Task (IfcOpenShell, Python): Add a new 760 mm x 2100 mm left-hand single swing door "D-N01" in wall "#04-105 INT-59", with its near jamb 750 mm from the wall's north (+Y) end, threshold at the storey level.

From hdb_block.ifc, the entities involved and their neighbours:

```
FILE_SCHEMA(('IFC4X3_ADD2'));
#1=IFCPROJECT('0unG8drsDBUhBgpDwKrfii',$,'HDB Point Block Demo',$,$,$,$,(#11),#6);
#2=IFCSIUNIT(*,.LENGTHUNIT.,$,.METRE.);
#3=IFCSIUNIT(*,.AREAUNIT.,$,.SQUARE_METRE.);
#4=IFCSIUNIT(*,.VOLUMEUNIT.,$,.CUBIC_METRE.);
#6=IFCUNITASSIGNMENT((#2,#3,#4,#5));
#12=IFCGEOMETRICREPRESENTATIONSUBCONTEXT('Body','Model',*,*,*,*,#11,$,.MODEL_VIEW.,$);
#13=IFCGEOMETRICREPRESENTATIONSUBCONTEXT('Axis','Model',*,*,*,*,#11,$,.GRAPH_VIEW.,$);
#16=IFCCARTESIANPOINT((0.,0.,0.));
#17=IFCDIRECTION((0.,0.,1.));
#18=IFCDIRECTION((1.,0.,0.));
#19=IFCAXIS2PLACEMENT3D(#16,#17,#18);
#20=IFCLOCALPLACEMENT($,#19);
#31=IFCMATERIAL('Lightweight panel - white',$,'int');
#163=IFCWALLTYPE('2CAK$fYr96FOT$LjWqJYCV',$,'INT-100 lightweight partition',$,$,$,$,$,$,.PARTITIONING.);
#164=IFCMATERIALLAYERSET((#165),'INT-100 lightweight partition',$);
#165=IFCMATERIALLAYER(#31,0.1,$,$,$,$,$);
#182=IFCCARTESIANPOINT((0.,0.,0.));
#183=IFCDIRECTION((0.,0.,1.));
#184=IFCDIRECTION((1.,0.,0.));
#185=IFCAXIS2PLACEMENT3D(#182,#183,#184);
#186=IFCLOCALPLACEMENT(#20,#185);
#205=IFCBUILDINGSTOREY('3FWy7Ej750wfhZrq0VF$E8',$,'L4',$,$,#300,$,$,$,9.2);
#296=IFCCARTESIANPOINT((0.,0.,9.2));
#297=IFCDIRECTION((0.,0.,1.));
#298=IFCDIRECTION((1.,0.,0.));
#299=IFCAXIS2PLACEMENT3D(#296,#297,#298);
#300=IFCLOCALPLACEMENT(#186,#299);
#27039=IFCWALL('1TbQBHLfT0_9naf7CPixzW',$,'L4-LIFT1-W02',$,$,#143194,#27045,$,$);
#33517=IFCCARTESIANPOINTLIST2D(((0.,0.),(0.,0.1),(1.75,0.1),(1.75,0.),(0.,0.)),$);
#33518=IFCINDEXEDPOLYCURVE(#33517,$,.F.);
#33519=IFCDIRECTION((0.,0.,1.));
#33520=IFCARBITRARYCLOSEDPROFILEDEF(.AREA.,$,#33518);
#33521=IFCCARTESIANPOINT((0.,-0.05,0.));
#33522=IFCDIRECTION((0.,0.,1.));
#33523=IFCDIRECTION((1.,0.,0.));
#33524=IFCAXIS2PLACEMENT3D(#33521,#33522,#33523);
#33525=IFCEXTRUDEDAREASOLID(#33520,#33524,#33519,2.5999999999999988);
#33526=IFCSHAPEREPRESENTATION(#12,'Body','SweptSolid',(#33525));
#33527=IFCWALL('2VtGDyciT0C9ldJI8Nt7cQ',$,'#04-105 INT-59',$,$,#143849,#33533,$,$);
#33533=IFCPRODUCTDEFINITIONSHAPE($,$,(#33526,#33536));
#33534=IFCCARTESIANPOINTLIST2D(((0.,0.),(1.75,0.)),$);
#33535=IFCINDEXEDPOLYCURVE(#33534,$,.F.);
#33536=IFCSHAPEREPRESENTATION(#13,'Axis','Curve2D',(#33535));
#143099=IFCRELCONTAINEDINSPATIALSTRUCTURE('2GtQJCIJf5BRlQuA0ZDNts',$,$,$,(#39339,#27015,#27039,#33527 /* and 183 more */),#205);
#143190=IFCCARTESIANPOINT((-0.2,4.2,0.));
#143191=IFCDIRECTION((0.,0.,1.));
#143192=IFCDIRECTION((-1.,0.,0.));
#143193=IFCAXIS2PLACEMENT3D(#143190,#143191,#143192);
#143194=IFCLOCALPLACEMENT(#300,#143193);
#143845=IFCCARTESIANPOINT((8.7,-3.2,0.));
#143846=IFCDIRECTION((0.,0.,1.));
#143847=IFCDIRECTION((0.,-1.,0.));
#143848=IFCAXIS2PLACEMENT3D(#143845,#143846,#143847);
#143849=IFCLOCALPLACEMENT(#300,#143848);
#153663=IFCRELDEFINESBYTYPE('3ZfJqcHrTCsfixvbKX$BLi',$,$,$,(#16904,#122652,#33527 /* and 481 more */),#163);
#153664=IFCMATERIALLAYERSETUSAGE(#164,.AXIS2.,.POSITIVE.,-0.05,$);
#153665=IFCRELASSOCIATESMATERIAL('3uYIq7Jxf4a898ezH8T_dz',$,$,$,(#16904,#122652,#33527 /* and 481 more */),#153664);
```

```python
import numpy as np
import ifcopenshell
import ifcopenshell.api.feature
import ifcopenshell.api.geometry
import ifcopenshell.api.root
import ifcopenshell.api.spatial
import ifcopenshell.geom
import ifcopenshell.util.element
import ifcopenshell.util.placement
import ifcopenshell.util.representation
import ifcopenshell.util.shape
import ifcopenshell.util.unit

model = ifcopenshell.open("hdb_block.ifc")
unit_scale = ifcopenshell.util.unit.calculate_unit_scale(model)
settings = ifcopenshell.geom.settings()


def volume(element):
    """Net volume in cubic metres, openings subtracted."""
    shape = ifcopenshell.geom.create_shape(settings, element)
    return ifcopenshell.util.shape.get_volume(shape.geometry)


wall = model.by_guid("2VtGDyciT0C9ldJI8Nt7cQ")
storey = ifcopenshell.util.element.get_container(wall, ifc_class="IfcBuildingStorey")
context = ifcopenshell.util.representation.get_context(model, "Model", "Body", "MODEL_VIEW")
before = volume(wall)

width, height, from_end, sill = 0.76, 2.1, 0.75, 0.0  # metres

# The wall runs along its own X axis, and the end named is its -X end.
wall_shape = ifcopenshell.geom.create_shape(settings, wall)
x, y, z = ifcopenshell.util.shape.get_vertices(wall_shape.geometry).T
start = x.min() + from_end
face, thickness = float(y.min()), float(y.max() - y.min())
wall_matrix = ifcopenshell.util.placement.get_local_placement(wall.ObjectPlacement)
level = ifcopenshell.util.placement.get_local_placement(storey.ObjectPlacement)[2, 3]


def in_wall(x, y):
    """Placement at x, y metres in the wall's axes, at sill height."""
    matrix = wall_matrix.copy()
    matrix[:, 3] = wall_matrix @ np.array([x / unit_scale, y / unit_scale, 0.0, 1.0])
    matrix[2, 3] = level + sill / unit_scale
    return matrix


# Opening: a box that overshoots both wall faces by 50 mm.
opening = ifcopenshell.api.root.create_entity(model, ifc_class="IfcOpeningElement", predefined_type="OPENING")
box = ifcopenshell.api.geometry.add_wall_representation(
    model, context=context, length=width, height=height, thickness=thickness + 0.1
)
ifcopenshell.api.geometry.assign_representation(model, product=opening, representation=box)
ifcopenshell.api.geometry.edit_object_placement(model, product=opening, matrix=in_wall(start, face - 0.05), is_si=False)
ifcopenshell.api.feature.add_feature(model, feature=opening, element=wall)

door = ifcopenshell.api.root.create_entity(model, ifc_class="IfcDoor", name="D-N01", predefined_type="DOOR")
door.OverallWidth, door.OverallHeight = width / unit_scale, height / unit_scale
door.OperationType = "SINGLE_SWING_LEFT"
body = ifcopenshell.api.geometry.add_door_representation(
    model,
    context=context,
    overall_width=door.OverallWidth,
    overall_height=door.OverallHeight,
    operation_type="SINGLE_SWING_LEFT",
    lining_properties={"LiningDepth": thickness / unit_scale, "ThresholdDepth": thickness / unit_scale},
)
ifcopenshell.api.geometry.assign_representation(model, product=door, representation=body)
ifcopenshell.api.spatial.assign_container(model, products=[door], relating_structure=storey)
ifcopenshell.api.feature.add_filling(model, opening=opening, element=door)

# The lining spans the wall, so the door starts at the wall face.
ifcopenshell.api.geometry.edit_object_placement(model, product=door, matrix=in_wall(start, face), is_si=False)

after = volume(wall)

print(f"wall volume {before:.3f} -> {after:.3f} m3")

model.write("hdb_block_updated.ifc")
```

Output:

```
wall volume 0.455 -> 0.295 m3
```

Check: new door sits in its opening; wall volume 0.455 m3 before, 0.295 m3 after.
